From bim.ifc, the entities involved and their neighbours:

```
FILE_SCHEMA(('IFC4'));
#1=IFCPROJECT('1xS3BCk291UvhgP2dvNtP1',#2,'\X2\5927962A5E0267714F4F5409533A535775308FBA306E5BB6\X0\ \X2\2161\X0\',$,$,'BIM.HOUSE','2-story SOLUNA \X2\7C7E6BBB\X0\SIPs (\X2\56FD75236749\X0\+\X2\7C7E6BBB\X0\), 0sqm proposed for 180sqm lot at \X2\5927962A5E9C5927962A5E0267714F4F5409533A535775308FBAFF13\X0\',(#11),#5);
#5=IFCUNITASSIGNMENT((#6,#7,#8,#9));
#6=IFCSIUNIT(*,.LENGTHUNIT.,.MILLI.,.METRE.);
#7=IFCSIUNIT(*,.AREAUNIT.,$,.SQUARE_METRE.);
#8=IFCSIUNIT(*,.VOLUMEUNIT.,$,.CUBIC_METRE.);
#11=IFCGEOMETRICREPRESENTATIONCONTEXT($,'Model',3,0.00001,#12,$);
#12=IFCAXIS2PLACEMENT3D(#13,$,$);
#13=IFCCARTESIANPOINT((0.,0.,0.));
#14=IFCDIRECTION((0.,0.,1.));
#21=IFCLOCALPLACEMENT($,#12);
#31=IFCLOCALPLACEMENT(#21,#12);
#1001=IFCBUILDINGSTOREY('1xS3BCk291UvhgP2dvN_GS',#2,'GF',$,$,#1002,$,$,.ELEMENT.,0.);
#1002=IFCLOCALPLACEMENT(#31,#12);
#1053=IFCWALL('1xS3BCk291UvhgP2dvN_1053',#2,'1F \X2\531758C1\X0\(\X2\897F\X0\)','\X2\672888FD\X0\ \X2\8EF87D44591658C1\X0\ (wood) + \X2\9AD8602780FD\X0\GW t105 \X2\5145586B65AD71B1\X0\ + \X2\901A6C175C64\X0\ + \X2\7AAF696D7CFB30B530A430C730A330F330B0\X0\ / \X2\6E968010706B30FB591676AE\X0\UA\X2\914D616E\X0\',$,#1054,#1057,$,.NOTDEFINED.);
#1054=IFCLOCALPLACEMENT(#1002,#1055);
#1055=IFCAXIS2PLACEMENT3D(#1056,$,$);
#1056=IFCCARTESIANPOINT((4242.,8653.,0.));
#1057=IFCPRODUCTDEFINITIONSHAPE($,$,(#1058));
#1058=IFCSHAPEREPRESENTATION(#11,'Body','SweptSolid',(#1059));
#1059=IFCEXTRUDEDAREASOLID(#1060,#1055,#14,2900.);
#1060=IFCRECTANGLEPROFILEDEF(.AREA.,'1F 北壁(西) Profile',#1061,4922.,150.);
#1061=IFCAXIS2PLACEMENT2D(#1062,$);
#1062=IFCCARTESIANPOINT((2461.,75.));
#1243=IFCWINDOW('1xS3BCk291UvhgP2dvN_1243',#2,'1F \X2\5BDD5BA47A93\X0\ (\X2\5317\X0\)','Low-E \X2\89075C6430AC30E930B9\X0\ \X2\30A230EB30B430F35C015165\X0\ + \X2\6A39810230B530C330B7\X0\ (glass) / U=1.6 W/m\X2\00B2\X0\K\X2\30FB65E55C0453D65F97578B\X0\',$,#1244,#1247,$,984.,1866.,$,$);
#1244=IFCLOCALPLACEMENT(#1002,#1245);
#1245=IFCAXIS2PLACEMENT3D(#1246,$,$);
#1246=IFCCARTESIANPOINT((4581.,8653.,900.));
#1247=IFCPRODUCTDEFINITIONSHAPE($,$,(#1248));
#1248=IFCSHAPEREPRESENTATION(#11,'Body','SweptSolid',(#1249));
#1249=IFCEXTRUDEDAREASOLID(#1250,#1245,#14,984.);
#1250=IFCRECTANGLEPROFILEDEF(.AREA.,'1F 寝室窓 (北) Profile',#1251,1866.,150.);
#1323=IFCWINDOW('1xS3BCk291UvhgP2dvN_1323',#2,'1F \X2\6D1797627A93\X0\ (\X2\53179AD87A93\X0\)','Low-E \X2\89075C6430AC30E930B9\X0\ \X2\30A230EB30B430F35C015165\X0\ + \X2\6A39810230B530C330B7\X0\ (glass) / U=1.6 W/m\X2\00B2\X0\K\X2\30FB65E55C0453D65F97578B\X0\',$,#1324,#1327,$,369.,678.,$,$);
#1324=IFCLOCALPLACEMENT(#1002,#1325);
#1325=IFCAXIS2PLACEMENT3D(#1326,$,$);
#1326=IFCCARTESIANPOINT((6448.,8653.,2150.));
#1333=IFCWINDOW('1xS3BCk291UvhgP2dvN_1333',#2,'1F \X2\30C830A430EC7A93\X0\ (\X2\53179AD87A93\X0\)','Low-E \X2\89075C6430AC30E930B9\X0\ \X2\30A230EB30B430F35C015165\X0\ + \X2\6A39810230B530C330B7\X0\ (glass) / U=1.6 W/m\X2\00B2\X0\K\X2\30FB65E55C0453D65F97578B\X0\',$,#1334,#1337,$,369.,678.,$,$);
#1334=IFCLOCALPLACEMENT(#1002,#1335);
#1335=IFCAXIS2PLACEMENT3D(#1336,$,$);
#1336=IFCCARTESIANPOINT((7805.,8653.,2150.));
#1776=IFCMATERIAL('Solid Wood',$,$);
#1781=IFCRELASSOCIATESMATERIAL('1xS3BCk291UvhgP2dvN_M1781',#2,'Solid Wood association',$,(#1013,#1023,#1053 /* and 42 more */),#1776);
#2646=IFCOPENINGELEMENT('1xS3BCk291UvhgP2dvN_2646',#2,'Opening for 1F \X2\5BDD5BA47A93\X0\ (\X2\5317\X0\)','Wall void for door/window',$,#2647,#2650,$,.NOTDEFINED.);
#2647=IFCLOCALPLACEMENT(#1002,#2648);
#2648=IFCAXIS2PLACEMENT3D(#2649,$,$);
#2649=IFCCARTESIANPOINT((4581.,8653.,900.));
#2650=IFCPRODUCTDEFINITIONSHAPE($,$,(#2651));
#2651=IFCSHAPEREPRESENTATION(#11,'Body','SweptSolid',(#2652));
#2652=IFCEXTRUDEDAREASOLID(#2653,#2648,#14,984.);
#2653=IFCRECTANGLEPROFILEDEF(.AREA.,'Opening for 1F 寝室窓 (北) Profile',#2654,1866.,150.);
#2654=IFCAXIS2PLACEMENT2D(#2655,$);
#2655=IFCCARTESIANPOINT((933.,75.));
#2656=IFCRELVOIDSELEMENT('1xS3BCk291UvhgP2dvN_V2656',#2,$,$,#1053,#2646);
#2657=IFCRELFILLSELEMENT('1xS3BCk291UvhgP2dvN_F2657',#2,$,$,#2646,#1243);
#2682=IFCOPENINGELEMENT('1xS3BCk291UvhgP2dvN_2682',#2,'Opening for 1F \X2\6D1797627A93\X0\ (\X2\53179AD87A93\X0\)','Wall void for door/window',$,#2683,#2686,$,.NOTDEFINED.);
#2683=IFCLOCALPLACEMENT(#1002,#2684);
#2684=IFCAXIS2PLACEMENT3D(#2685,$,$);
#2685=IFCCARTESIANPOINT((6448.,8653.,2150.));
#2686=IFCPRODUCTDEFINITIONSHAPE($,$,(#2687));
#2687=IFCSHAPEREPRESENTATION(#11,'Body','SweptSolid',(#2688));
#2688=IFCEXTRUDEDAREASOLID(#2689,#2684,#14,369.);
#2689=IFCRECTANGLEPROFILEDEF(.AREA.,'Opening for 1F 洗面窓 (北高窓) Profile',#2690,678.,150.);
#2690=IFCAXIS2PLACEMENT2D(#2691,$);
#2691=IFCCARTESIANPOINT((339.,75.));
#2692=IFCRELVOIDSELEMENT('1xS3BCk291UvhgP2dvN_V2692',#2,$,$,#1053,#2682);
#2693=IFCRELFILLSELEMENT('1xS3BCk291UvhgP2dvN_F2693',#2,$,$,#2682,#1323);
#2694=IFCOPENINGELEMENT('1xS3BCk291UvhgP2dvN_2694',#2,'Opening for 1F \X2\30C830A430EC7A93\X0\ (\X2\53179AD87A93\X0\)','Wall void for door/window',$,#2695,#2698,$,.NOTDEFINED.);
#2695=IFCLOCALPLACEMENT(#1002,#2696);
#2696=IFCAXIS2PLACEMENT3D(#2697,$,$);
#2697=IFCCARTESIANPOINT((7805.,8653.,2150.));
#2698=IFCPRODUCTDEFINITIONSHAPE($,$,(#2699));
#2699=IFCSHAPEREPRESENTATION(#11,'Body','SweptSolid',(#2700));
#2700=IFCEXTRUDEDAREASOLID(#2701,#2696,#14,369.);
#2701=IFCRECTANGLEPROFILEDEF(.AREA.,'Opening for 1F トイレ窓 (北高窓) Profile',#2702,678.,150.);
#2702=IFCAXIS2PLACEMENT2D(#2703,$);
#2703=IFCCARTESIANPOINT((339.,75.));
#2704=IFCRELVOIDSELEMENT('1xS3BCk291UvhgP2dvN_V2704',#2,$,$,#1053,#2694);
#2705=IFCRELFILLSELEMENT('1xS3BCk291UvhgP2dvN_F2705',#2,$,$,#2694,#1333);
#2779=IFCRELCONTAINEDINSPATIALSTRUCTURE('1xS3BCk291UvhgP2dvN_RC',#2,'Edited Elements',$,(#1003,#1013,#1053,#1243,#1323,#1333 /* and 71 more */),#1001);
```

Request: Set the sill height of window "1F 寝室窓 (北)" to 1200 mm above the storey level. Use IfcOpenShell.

```python
import numpy as np
import ifcopenshell
import ifcopenshell.api.geometry
import ifcopenshell.geom
import ifcopenshell.util.element
import ifcopenshell.util.placement
import ifcopenshell.util.shape
import ifcopenshell.util.unit

model = ifcopenshell.open("bim.ifc")
unit_scale = ifcopenshell.util.unit.calculate_unit_scale(model)

window = model.by_id(1243)
opening = window.FillsVoids[0].RelatingOpeningElement
storey = ifcopenshell.util.element.get_container(window, ifc_class="IfcBuildingStorey")
level = ifcopenshell.util.placement.get_local_placement(storey.ObjectPlacement)[2, 3]

# The opening's origin need not be at the sill, so measure its lowest point.
shape = ifcopenshell.geom.create_shape(ifcopenshell.geom.settings(), opening)
bottom = ifcopenshell.util.shape.get_shape_bottom_elevation(shape, shape.geometry) / unit_scale
dz = level + 1.2 / unit_scale - bottom

shift = np.array([0.0, 0.0, dz])
# The window is not placed relative to its opening, so move both.
for product in (opening, window):
    matrix = ifcopenshell.util.placement.get_local_placement(product.ObjectPlacement)
    matrix[:3, 3] += shift
    ifcopenshell.api.geometry.edit_object_placement(model, product=product, matrix=matrix, is_si=False)

print(f"moved by {dz * unit_scale:+.3f} m")

model.write("bim_rev.ifc")
```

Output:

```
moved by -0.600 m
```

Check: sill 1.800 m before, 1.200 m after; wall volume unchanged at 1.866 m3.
